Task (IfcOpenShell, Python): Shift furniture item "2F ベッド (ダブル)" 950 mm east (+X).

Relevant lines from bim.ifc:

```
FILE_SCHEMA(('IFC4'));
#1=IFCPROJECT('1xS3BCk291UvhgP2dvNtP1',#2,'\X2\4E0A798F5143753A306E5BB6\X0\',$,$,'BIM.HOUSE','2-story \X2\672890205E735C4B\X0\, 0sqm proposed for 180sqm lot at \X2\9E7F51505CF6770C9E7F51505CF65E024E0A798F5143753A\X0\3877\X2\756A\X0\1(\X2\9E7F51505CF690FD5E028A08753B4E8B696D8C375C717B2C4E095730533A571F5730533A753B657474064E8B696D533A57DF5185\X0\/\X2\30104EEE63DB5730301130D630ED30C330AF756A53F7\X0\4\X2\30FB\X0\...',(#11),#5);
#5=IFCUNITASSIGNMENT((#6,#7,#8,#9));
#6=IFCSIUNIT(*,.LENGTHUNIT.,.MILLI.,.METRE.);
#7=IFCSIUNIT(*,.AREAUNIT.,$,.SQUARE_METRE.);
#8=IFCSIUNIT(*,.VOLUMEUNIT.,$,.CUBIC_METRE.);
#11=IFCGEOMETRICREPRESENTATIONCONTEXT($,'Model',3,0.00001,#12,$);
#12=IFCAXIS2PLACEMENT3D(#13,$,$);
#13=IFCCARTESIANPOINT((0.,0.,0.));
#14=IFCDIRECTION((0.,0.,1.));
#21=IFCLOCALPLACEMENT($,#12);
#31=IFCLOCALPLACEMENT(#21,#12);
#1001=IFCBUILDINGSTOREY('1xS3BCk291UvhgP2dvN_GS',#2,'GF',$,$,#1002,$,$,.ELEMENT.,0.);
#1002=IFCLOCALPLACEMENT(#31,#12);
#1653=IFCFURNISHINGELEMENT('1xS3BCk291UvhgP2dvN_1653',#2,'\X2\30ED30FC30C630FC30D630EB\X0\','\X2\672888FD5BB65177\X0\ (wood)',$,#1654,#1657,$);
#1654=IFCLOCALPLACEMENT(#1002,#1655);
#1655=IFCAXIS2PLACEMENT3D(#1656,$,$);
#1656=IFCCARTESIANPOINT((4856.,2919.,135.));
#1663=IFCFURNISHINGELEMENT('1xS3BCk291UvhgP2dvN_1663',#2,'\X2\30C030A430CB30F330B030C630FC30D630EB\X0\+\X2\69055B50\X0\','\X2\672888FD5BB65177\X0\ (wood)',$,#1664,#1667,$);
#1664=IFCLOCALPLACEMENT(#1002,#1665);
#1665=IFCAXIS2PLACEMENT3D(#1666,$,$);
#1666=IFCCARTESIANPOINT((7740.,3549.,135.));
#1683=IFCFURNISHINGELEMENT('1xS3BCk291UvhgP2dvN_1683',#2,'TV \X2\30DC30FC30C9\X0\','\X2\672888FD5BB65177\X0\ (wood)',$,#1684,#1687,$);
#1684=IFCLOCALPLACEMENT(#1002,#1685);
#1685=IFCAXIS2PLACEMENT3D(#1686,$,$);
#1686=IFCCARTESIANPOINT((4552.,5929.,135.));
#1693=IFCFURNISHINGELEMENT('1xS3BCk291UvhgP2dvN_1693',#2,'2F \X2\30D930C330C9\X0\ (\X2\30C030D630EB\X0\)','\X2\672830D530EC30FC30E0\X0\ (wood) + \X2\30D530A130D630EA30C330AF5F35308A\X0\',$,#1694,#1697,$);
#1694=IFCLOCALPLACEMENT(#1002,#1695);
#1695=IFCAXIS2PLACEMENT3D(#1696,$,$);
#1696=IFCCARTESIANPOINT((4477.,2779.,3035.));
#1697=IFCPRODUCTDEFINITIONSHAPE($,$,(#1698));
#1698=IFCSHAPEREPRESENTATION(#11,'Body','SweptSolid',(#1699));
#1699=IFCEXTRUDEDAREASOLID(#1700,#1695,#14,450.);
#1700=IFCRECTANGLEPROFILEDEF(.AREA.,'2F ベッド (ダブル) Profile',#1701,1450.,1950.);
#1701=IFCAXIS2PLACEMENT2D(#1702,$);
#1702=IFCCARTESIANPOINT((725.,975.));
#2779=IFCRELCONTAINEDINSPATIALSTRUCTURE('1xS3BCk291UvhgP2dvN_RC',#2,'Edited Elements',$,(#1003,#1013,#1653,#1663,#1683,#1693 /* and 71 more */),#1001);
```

```python
import ifcopenshell
import ifcopenshell.api.geometry
import ifcopenshell.util.placement
import ifcopenshell.util.unit

model = ifcopenshell.open("bim.ifc")
unit_scale = ifcopenshell.util.unit.calculate_unit_scale(model)

item = model.by_guid("1xS3BCk291UvhgP2dvN_1693")
matrix = ifcopenshell.util.placement.get_local_placement(item.ObjectPlacement)
matrix[0, 3] += 0.95 / unit_scale
ifcopenshell.api.geometry.edit_object_placement(model, product=item, matrix=matrix, is_si=False)

print(ifcopenshell.util.placement.get_local_placement(item.ObjectPlacement).round(3) + 0.0)

model.write("bim_rev.ifc")
```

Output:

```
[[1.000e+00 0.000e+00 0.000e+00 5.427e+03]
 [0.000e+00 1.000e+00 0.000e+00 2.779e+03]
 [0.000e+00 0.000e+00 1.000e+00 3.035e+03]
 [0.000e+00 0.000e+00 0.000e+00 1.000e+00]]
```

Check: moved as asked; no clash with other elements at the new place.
